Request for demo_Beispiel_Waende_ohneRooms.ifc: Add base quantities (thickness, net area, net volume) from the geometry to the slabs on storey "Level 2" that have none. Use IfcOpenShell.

First a look at what the model holds.

```python
import ifcopenshell
import ifcopenshell.util.element
import ifcopenshell.util.unit

model = ifcopenshell.open("demo_Beispiel_Waende_ohneRooms.ifc")
print(model.schema)
for unit_type in ("LENGTHUNIT", "AREAUNIT", "VOLUMEUNIT"):
    print(unit_type, ifcopenshell.util.unit.calculate_unit_scale(model, unit_type))
storey = next(s for s in model.by_type("IfcBuildingStorey") if s.Name == "Level 2")
slabs = [e for e in ifcopenshell.util.element.get_decomposition(storey) if e.is_a("IfcSlab")]
for e in sorted(slabs, key=lambda e: e.id()):
    print(e.id(), e.is_a(), e.Name, list(ifcopenshell.util.element.get_psets(e, qtos_only=True)), sep=" | ")
```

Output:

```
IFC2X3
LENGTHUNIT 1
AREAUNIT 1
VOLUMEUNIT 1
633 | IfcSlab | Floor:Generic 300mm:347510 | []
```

```python
import ifcopenshell
import ifcopenshell.api.pset
import ifcopenshell.geom
import ifcopenshell.util.element
import ifcopenshell.util.shape
import ifcopenshell.util.unit

model = ifcopenshell.open("demo_Beispiel_Waende_ohneRooms.ifc")
unit_scale = ifcopenshell.util.unit.calculate_unit_scale(model)
area_scale = ifcopenshell.util.unit.calculate_unit_scale(model, "AREAUNIT")
volume_scale = ifcopenshell.util.unit.calculate_unit_scale(model, "VOLUMEUNIT")
settings = ifcopenshell.geom.settings()

storey = next(s for s in model.by_type("IfcBuildingStorey") if s.Name == "Level 2")
slabs = [e for e in ifcopenshell.util.element.get_decomposition(storey) if e.is_a("IfcSlab")]

for e in sorted(slabs, key=lambda e: e.id()):
    if ifcopenshell.util.element.get_psets(e, qtos_only=True, should_inherit=False):
        continue
    # Geometry comes back in metres, in the element's own axes.
    shape = ifcopenshell.geom.create_shape(settings, e)
    values = {
        "Width": ifcopenshell.util.shape.get_z(shape.geometry) / unit_scale,
        "NetArea": ifcopenshell.util.shape.get_footprint_area(shape.geometry) / area_scale,
        "NetVolume": ifcopenshell.util.shape.get_volume(shape.geometry) / volume_scale,
    }
    qto = ifcopenshell.api.pset.add_qto(model, product=e, name="BaseQuantities")
    ifcopenshell.api.pset.edit_qto(model, qto=qto, properties=values)
    print(e.id(), {k: round(v, 3) for k, v in values.items()})

model.write("demo_Beispiel_Waende_ohneRooms_edited.ifc")
```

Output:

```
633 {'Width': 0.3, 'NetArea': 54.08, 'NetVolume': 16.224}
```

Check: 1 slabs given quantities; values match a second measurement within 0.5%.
